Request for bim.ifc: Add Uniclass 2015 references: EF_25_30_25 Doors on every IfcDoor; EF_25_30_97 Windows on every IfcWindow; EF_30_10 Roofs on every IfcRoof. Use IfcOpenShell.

First a look at what the model holds.

```python
import ifcopenshell

model = ifcopenshell.open("bim.ifc")
print(model.schema)
print("classifications:", [c.Name for c in model.by_type("IfcClassification")])
for ifc_class in ("IfcDoor", "IfcRoof", "IfcStair", "IfcWall", "IfcWindow"):
    print(ifc_class, len(model.by_type(ifc_class)))
```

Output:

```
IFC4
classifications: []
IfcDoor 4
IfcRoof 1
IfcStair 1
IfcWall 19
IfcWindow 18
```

```python
import ifcopenshell
import ifcopenshell.api.classification

model = ifcopenshell.open("bim.ifc")

system = ifcopenshell.api.classification.add_classification(model, classification="Uniclass 2015")

codes = {
    "IfcDoor": ("EF_25_30_25", "Doors"),
    "IfcWindow": ("EF_25_30_97", "Windows"),
    "IfcRoof": ("EF_30_10", "Roofs"),
}
for ifc_class, (code, name) in codes.items():
    products = model.by_type(ifc_class)
    ifcopenshell.api.classification.add_reference(
        model, products=products, classification=system, identification=code, name=name
    )
    print(code, len(products))

model.write("bim-out.ifc")
```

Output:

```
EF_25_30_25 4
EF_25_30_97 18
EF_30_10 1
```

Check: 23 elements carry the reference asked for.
